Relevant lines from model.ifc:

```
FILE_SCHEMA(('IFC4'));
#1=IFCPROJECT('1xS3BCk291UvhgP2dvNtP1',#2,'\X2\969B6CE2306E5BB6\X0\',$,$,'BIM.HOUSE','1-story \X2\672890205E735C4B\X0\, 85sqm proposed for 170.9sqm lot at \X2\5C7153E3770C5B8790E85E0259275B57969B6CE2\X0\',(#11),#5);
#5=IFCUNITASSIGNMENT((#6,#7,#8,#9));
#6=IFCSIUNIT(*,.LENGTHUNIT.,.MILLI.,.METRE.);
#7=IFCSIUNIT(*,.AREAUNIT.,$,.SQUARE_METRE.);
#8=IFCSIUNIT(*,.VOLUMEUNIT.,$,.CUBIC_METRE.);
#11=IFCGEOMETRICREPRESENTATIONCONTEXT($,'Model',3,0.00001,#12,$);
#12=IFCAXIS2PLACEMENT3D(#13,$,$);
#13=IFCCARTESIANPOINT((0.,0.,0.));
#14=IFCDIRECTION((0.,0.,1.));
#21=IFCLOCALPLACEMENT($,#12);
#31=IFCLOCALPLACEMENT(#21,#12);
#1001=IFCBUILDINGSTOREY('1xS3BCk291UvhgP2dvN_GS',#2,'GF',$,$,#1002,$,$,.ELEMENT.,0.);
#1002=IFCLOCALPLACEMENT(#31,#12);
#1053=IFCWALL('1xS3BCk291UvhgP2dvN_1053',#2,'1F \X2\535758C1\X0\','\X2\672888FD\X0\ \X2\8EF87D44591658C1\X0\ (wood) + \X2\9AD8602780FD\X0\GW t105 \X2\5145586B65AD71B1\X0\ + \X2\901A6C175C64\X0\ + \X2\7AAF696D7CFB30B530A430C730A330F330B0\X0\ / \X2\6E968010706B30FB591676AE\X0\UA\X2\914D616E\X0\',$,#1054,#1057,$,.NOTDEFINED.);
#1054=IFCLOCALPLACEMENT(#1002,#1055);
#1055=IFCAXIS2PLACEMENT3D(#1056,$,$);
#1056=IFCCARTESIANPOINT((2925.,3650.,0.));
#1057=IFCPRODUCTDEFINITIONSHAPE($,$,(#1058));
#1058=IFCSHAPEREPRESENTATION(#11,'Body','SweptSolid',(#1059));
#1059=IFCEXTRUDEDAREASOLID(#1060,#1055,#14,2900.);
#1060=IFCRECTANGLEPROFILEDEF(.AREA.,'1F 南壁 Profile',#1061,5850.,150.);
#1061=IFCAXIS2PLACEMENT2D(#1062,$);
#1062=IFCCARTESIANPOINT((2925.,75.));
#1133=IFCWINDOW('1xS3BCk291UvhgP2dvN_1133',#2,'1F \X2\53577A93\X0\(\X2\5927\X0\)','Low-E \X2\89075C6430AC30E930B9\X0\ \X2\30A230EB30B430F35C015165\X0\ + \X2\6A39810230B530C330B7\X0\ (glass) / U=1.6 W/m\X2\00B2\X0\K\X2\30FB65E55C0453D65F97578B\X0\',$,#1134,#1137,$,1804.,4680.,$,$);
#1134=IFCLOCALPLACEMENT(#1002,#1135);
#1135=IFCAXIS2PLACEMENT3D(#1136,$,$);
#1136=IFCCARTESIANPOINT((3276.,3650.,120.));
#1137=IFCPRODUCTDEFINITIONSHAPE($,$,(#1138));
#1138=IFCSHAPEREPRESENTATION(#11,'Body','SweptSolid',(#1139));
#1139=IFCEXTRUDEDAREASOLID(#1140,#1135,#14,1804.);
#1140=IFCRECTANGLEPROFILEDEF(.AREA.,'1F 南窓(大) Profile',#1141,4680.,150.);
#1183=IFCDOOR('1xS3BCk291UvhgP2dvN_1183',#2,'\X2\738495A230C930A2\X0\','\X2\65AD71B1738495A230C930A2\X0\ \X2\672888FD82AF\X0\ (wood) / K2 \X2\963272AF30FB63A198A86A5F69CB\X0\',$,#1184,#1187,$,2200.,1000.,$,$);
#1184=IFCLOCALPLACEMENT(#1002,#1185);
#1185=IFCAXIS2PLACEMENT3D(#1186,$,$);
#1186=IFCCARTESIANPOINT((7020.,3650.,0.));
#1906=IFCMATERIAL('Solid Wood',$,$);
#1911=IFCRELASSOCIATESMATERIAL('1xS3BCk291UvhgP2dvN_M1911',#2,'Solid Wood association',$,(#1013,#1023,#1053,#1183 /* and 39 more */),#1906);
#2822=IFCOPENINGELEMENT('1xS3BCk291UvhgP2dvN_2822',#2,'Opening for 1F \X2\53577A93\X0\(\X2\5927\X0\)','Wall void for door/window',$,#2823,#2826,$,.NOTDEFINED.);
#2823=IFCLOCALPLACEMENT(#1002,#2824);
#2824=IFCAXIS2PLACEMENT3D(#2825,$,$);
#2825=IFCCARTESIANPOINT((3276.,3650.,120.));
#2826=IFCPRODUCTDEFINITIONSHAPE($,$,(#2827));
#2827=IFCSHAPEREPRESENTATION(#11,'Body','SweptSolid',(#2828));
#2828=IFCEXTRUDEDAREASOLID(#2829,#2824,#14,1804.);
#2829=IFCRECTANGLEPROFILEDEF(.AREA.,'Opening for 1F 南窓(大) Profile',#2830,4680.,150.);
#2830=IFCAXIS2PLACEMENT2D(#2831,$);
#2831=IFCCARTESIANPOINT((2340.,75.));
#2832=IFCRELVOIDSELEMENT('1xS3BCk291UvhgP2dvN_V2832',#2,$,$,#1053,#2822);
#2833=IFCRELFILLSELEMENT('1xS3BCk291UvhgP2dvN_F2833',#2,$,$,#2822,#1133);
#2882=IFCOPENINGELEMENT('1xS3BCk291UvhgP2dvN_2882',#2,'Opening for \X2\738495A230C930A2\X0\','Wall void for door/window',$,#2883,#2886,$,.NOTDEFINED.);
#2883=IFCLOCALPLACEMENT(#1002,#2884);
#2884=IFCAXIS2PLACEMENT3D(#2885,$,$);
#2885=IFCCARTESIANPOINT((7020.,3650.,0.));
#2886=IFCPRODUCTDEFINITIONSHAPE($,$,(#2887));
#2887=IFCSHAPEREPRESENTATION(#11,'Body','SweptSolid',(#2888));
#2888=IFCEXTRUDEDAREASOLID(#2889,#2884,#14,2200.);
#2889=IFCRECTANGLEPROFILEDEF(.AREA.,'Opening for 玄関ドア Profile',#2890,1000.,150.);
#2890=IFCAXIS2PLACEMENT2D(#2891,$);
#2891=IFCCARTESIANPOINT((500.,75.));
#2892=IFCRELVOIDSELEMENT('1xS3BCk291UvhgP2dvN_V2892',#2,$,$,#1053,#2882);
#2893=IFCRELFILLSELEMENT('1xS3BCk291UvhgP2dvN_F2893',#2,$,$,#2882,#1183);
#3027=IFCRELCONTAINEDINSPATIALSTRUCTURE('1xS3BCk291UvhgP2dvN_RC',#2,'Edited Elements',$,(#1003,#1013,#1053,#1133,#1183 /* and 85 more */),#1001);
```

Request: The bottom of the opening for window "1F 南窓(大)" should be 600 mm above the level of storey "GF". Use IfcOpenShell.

```python
import numpy as np
import ifcopenshell
import ifcopenshell.api.geometry
import ifcopenshell.geom
import ifcopenshell.util.element
import ifcopenshell.util.placement
import ifcopenshell.util.shape
import ifcopenshell.util.unit

model = ifcopenshell.open("model.ifc")
unit_scale = ifcopenshell.util.unit.calculate_unit_scale(model)

window = model.by_id(1133)
opening = window.FillsVoids[0].RelatingOpeningElement
storey = ifcopenshell.util.element.get_container(window, ifc_class="IfcBuildingStorey")
level = ifcopenshell.util.placement.get_local_placement(storey.ObjectPlacement)[2, 3]

# The opening's origin need not be at the sill, so measure its lowest point.
shape = ifcopenshell.geom.create_shape(ifcopenshell.geom.settings(), opening)
bottom = ifcopenshell.util.shape.get_shape_bottom_elevation(shape, shape.geometry) / unit_scale
dz = level + 0.6 / unit_scale - bottom

shift = np.array([0.0, 0.0, dz])
# The window is not placed relative to its opening, so move both.
for product in (opening, window):
    matrix = ifcopenshell.util.placement.get_local_placement(product.ObjectPlacement)
    matrix[:3, 3] += shift
    ifcopenshell.api.geometry.edit_object_placement(model, product=product, matrix=matrix, is_si=False)

print(f"moved by {dz * unit_scale:+.3f} m")

model.write("model-out.ifc")
```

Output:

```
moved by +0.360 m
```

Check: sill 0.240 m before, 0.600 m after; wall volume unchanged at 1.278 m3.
